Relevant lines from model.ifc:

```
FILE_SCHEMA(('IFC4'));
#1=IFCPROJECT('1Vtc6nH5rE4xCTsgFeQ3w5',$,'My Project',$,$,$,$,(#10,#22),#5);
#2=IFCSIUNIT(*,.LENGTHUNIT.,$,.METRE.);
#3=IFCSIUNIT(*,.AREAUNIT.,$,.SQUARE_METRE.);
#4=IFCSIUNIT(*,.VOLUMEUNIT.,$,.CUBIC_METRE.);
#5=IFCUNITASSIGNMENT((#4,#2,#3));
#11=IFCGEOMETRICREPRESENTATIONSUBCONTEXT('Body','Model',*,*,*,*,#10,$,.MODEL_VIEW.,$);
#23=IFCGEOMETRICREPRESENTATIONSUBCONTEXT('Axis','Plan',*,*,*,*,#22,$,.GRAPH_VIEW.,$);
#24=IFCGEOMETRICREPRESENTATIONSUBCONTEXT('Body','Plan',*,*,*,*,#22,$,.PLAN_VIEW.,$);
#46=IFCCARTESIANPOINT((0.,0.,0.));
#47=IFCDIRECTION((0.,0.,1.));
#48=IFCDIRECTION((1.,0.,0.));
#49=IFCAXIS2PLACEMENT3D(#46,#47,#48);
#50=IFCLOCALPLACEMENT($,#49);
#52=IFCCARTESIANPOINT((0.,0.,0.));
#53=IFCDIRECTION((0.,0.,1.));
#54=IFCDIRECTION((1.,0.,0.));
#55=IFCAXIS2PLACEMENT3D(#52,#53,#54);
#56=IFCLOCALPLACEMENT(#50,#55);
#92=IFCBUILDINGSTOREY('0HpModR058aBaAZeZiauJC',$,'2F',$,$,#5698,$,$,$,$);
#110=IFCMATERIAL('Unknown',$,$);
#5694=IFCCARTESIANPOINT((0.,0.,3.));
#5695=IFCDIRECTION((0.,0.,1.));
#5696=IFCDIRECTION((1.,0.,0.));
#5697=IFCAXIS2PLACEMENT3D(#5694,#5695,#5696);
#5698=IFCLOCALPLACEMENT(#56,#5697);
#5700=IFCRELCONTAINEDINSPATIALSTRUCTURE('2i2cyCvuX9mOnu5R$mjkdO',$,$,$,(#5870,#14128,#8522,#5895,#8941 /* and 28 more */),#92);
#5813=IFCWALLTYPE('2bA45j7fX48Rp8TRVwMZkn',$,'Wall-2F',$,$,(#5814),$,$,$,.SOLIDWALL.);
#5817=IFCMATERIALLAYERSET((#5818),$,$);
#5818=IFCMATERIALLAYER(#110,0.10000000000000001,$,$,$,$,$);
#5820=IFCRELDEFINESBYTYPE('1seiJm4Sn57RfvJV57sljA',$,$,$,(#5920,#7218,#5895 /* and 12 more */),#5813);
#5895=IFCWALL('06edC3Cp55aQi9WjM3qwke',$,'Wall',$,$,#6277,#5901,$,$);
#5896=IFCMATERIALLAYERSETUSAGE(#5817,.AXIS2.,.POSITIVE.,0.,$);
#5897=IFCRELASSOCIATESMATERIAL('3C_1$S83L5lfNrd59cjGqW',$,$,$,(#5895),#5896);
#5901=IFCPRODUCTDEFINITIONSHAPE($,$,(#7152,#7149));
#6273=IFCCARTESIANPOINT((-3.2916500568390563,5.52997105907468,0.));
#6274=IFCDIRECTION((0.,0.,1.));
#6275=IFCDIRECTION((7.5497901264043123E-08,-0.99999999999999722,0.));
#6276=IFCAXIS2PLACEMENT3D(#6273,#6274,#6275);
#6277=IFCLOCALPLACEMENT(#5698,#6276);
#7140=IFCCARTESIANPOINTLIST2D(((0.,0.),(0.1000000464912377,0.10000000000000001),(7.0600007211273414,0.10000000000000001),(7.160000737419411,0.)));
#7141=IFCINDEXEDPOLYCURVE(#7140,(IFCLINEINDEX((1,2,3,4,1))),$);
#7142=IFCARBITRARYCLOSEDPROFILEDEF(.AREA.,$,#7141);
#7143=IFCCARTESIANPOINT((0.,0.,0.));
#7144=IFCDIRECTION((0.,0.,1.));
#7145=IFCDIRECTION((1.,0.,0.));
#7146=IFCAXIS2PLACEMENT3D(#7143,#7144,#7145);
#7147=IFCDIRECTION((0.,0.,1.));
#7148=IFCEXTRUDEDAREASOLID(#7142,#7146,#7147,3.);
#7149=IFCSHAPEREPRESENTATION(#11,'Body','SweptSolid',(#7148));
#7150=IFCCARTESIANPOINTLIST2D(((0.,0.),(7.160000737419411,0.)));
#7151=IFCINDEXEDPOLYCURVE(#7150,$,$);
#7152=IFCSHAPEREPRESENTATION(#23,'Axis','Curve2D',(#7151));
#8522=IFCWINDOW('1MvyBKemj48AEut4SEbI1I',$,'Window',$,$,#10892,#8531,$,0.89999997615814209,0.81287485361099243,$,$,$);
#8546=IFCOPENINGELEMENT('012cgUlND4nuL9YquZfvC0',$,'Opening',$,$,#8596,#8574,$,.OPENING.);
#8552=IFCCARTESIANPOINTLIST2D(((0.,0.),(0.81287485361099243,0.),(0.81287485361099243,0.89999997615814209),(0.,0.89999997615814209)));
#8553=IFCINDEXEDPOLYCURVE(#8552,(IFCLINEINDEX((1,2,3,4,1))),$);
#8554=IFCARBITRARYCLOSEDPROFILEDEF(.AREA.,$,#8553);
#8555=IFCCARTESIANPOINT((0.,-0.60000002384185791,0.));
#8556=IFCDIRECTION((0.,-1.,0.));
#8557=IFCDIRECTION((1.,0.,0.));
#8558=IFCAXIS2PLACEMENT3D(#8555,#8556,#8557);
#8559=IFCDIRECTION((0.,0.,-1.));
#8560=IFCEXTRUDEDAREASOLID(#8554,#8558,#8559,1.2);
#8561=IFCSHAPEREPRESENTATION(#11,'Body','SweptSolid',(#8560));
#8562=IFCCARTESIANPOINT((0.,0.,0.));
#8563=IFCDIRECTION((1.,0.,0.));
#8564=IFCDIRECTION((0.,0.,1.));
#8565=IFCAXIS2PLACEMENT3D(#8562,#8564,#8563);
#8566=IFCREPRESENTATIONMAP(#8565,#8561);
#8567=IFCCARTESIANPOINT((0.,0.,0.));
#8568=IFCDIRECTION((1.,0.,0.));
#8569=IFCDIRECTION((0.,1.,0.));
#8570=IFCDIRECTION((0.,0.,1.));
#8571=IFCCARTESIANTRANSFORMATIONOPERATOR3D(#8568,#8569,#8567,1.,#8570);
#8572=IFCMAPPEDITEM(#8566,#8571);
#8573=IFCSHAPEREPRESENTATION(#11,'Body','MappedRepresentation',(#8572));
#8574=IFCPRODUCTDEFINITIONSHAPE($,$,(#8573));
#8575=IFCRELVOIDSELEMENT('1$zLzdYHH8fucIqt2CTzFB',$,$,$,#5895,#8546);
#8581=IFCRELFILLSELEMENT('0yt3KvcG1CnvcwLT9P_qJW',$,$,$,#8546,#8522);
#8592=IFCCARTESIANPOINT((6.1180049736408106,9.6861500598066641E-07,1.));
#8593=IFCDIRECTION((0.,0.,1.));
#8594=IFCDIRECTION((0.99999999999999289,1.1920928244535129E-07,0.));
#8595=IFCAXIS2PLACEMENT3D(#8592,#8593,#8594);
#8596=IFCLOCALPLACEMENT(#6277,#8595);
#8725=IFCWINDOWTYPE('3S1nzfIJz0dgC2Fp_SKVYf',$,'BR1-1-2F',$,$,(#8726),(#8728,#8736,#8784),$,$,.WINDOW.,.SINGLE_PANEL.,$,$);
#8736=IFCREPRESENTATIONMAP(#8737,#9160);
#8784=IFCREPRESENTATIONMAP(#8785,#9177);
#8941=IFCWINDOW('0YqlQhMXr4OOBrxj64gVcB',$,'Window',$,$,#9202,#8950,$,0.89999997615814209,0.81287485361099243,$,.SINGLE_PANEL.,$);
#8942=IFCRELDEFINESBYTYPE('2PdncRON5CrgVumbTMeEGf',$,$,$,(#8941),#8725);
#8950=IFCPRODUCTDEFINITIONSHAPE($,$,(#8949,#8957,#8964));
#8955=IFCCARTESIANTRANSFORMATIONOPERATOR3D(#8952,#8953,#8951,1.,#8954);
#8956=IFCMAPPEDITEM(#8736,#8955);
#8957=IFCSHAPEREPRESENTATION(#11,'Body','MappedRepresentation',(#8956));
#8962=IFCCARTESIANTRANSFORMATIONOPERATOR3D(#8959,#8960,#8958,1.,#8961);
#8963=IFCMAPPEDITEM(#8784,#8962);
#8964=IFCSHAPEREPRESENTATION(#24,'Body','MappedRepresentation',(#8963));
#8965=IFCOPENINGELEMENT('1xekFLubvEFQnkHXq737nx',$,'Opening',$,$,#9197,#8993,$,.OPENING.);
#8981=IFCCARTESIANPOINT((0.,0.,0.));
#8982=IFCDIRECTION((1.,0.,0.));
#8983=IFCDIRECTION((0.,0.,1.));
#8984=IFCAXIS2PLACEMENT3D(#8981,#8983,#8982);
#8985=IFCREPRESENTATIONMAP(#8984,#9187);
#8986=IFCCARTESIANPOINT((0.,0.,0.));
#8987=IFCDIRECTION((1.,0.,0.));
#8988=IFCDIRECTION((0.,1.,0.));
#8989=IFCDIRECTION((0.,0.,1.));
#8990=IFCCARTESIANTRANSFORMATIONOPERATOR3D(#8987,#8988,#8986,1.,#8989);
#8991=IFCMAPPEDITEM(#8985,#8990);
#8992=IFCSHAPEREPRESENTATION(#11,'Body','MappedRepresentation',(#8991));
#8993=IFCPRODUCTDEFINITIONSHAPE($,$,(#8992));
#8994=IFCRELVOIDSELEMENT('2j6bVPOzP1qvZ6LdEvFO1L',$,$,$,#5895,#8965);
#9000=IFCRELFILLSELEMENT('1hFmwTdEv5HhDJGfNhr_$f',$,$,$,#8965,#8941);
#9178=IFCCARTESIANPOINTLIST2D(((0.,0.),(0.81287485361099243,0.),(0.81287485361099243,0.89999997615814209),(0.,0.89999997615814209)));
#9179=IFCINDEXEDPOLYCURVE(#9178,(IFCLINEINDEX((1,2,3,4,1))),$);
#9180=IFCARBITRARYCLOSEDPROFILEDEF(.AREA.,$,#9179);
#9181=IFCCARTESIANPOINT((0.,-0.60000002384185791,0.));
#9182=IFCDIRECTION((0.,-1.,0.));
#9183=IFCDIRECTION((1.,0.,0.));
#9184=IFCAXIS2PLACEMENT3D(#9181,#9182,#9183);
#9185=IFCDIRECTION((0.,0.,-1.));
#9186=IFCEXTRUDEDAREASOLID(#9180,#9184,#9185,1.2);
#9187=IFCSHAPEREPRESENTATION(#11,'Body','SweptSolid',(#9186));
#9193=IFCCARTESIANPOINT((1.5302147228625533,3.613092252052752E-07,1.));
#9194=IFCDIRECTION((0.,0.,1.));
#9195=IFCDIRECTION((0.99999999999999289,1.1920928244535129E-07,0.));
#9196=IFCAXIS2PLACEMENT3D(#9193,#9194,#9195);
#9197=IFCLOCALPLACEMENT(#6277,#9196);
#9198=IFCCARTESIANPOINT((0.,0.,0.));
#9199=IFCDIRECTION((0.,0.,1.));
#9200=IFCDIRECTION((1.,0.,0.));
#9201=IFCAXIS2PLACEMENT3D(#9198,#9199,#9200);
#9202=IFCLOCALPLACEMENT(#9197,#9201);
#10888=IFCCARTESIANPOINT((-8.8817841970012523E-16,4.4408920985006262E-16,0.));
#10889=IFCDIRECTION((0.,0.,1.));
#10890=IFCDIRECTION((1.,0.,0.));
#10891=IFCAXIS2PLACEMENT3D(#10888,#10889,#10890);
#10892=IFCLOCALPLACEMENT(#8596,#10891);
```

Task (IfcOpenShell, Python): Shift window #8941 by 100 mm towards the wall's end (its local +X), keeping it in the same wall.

```python
import ifcopenshell
import ifcopenshell.api.geometry
import ifcopenshell.util.placement
import ifcopenshell.util.unit

model = ifcopenshell.open("model.ifc")
unit_scale = ifcopenshell.util.unit.calculate_unit_scale(model)

window = model.by_guid("0YqlQhMXr4OOBrxj64gVcB")
opening = window.FillsVoids[0].RelatingOpeningElement
wall = opening.VoidsElements[0].RelatingBuildingElement

wall_matrix = ifcopenshell.util.placement.get_local_placement(wall.ObjectPlacement)
shift = wall_matrix[:3, 0] * 0.1 / unit_scale
before = ifcopenshell.util.placement.get_local_placement(window.ObjectPlacement)[:3, 3].copy()

# The window is placed relative to its opening, so it follows when the opening moves.
matrix = ifcopenshell.util.placement.get_local_placement(opening.ObjectPlacement)
matrix[:3, 3] += shift
ifcopenshell.api.geometry.edit_object_placement(
    model, product=opening, matrix=matrix, is_si=False, should_transform_children=True
)

after = ifcopenshell.util.placement.get_local_placement(window.ObjectPlacement)[:3, 3]
print("window moved by", (after - before).round(3) + 0.0)

model.write("model_v2.ifc")
```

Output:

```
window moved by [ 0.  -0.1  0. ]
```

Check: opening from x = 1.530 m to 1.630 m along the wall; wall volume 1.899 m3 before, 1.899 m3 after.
